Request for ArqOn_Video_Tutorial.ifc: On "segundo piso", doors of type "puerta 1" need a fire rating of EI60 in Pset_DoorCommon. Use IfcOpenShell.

First a look at what the model holds.

```python
import ifcopenshell
import ifcopenshell.util.element

model = ifcopenshell.open("ArqOn_Video_Tutorial.ifc")
print(model.schema)
storey = next(s for s in model.by_type("IfcBuildingStorey") if s.Name == "segundo piso")
doors = [e for e in ifcopenshell.util.element.get_decomposition(storey) if e.is_a("IfcDoor")]
seen = {}
for e in doors:
    element_type = ifcopenshell.util.element.get_type(e)
    key = (element_type.Name if element_type != e and element_type else None, ifcopenshell.util.element.get_pset(e, "Pset_DoorCommon", "FireRating"))
    seen[key] = seen.get(key, 0) + 1
for (name, value), count in sorted(seen.items(), key=str):
    print(count, "x", name, "|", value)
```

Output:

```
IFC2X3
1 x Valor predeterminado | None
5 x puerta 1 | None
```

```python
import ifcopenshell
import ifcopenshell.api.pset
import ifcopenshell.util.element

model = ifcopenshell.open("ArqOn_Video_Tutorial.ifc")

storey = next(s for s in model.by_type("IfcBuildingStorey") if s.Name == "segundo piso")
doors = [e for e in ifcopenshell.util.element.get_decomposition(storey) if e.is_a("IfcDoor")]

count = 0
for e in doors:
    element_type = ifcopenshell.util.element.get_type(e)
    if element_type in (None, e) or element_type.Name != "puerta 1":
        continue
    # add_pset returns the element's existing set when there is one.
    pset = ifcopenshell.api.pset.add_pset(model, product=e, name="Pset_DoorCommon")
    ifcopenshell.api.pset.edit_pset(model, pset=pset, properties={"FireRating": "EI60"})
    count += 1

print(count, "doors updated")

model.write("ArqOn_Video_Tutorial_edited.ifc")
```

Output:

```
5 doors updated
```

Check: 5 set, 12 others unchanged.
